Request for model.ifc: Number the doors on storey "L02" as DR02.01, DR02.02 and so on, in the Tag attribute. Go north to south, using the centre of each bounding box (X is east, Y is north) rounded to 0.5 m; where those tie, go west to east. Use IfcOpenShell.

First a look at what the model holds.

```python
import ifcopenshell
import ifcopenshell.util.element
import ifcopenshell.util.placement

model = ifcopenshell.open("model.ifc")
print(model.schema)
storey = next(s for s in model.by_type("IfcBuildingStorey") if s.Name == "L02")
doors = [e for e in ifcopenshell.util.element.get_decomposition(storey) if e.is_a("IfcDoor")]
for e in sorted(doors, key=lambda e: e.id()):
    origin = ifcopenshell.util.placement.get_local_placement(e.ObjectPlacement)[:3, 3]
    print(e.id(), e.Tag, e.Name, origin.round(2) + 0.0, sep=" | ")
```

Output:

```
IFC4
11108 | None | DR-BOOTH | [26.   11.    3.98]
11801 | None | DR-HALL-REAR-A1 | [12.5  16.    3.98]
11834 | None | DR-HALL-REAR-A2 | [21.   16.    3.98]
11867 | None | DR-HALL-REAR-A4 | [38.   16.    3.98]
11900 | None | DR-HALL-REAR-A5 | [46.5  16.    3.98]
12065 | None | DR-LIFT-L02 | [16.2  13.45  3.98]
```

```python
import ifcopenshell
import ifcopenshell.geom
import ifcopenshell.util.element
import ifcopenshell.util.shape

model = ifcopenshell.open("model.ifc")
settings = ifcopenshell.geom.settings()
settings.set("use-world-coords", True)


def centre(element):
    shape = ifcopenshell.geom.create_shape(settings, element)
    return ifcopenshell.util.shape.get_bbox_centroid(shape.geometry)


storey = next(s for s in model.by_type("IfcBuildingStorey") if s.Name == "L02")
doors = [e for e in ifcopenshell.util.element.get_decomposition(storey) if e.is_a("IfcDoor")]

# Insertion points can sit at a corner or the storey origin, so sort by the geometry (in metres).
centres = {e: centre(e) for e in doors}
doors.sort(key=lambda e: (-round(centres[e][1] / 0.5), centres[e][0]))

for i, e in enumerate(doors, start=1):
    number = f"DR02.{i:02d}"
    e.Tag = number
    print(e.id(), number)

model.write("model_v2.ifc")
```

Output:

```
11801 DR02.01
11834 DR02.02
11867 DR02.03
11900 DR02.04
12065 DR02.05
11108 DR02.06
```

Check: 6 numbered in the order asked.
